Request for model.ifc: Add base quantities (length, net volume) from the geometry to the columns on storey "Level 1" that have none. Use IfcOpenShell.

First a look at what the model holds.

```python
import ifcopenshell
import ifcopenshell.util.element
import ifcopenshell.util.unit

model = ifcopenshell.open("model.ifc")
print(model.schema)
for unit_type in ("LENGTHUNIT", "AREAUNIT", "VOLUMEUNIT"):
    print(unit_type, ifcopenshell.util.unit.calculate_unit_scale(model, unit_type))
storey = next(s for s in model.by_type("IfcBuildingStorey") if s.Name == "Level 1")
columns = [e for e in ifcopenshell.util.element.get_decomposition(storey) if e.is_a("IfcColumn")]
for e in sorted(columns, key=lambda e: e.id()):
    print(e.id(), e.is_a(), e.Name, list(ifcopenshell.util.element.get_psets(e, qtos_only=True)), sep=" | ")
```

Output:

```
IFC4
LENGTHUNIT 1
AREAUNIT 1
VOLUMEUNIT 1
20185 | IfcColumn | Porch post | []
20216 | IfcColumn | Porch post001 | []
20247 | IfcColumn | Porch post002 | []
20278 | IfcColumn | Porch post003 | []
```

```python
import ifcopenshell
import ifcopenshell.api.pset
import ifcopenshell.geom
import ifcopenshell.util.element
import ifcopenshell.util.shape
import ifcopenshell.util.unit

model = ifcopenshell.open("model.ifc")
unit_scale = ifcopenshell.util.unit.calculate_unit_scale(model)
volume_scale = ifcopenshell.util.unit.calculate_unit_scale(model, "VOLUMEUNIT")
settings = ifcopenshell.geom.settings()

storey = next(s for s in model.by_type("IfcBuildingStorey") if s.Name == "Level 1")
columns = [e for e in ifcopenshell.util.element.get_decomposition(storey) if e.is_a("IfcColumn")]

for e in sorted(columns, key=lambda e: e.id()):
    if ifcopenshell.util.element.get_psets(e, qtos_only=True, should_inherit=False):
        continue
    # Geometry comes back in metres, in the element's own axes.
    shape = ifcopenshell.geom.create_shape(settings, e)
    values = {
        "Length": ifcopenshell.util.shape.get_z(shape.geometry) / unit_scale,
        "NetVolume": ifcopenshell.util.shape.get_volume(shape.geometry) / volume_scale,
    }
    qto = ifcopenshell.api.pset.add_qto(model, product=e, name="Qto_ColumnBaseQuantities")
    ifcopenshell.api.pset.edit_qto(model, qto=qto, properties=values)
    print(e.id(), {k: round(v, 3) for k, v in values.items()})

model.write("model-out.ifc")
```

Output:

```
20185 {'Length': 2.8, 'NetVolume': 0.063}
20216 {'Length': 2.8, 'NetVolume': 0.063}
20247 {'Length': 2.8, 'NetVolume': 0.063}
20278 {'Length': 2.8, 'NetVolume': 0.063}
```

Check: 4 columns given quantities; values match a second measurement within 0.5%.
